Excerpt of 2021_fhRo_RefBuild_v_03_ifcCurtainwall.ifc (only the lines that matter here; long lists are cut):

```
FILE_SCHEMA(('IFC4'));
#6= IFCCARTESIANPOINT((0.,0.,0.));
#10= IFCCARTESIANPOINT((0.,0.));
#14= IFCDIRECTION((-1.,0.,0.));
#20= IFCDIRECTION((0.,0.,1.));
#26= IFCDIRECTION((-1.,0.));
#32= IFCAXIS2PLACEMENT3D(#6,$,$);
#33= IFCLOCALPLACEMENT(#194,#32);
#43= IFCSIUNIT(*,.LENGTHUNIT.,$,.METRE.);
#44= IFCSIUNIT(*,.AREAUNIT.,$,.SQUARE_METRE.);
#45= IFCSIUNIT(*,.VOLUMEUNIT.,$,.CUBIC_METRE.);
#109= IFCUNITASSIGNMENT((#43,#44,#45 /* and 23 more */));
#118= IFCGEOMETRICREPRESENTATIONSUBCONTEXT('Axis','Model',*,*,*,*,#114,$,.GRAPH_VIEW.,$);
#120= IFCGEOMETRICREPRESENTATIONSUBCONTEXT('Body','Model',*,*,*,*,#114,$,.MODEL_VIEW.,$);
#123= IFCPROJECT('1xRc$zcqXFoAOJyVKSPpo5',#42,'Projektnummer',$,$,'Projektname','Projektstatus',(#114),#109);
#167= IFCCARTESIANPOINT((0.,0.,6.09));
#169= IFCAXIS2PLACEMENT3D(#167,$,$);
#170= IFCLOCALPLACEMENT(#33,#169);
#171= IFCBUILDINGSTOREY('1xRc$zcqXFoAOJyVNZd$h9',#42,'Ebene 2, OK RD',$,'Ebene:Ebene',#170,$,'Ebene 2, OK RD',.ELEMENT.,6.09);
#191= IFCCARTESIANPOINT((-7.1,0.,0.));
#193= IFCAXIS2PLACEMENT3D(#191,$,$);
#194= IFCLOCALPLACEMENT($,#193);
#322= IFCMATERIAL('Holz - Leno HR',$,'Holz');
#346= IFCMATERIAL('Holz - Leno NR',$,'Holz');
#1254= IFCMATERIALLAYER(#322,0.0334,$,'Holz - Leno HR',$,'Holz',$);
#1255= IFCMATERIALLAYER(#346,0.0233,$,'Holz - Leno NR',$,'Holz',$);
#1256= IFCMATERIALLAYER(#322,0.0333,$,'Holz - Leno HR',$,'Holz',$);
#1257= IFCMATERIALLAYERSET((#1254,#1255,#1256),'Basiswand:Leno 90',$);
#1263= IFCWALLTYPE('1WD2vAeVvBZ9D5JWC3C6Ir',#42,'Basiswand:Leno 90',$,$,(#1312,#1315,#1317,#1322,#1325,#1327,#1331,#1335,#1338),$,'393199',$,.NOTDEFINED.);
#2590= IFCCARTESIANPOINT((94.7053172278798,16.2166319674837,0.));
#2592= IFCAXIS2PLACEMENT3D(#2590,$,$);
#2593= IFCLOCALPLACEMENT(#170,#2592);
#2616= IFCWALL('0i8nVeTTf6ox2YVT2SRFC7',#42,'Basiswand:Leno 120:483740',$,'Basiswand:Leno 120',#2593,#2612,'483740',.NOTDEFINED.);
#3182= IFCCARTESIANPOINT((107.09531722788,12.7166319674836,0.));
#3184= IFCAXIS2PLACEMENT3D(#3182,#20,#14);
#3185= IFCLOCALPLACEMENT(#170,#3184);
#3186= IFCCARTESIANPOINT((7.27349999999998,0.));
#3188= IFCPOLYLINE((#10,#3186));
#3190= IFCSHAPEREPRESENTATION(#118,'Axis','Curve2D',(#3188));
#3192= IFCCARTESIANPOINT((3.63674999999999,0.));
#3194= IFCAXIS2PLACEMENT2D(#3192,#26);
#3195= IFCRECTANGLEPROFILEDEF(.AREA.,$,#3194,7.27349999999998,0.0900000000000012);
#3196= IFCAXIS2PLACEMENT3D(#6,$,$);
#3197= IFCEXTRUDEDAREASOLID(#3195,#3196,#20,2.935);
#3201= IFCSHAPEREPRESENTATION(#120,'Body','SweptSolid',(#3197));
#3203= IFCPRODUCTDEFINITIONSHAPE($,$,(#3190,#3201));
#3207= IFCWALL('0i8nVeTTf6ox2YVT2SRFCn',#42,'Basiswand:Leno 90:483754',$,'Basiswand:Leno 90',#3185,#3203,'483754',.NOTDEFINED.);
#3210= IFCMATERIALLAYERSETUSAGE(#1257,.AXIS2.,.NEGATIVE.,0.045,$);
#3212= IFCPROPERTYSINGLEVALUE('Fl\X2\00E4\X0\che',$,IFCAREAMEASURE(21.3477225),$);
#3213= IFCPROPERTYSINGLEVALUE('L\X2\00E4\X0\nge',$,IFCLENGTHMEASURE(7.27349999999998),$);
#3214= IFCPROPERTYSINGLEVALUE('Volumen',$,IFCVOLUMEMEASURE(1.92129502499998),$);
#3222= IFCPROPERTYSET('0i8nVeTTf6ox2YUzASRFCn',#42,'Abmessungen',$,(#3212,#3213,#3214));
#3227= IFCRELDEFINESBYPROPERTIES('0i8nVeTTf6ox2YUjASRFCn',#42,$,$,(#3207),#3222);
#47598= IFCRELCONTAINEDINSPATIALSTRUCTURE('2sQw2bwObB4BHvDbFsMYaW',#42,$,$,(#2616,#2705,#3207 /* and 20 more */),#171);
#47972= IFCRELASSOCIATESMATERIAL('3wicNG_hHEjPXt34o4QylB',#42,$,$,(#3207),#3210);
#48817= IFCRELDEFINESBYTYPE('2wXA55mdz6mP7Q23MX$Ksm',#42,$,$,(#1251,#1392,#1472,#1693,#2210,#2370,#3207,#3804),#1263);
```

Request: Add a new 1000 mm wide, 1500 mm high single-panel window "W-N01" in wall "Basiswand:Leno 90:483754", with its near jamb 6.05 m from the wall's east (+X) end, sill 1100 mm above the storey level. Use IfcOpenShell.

```python
import numpy as np
import ifcopenshell
import ifcopenshell.api.feature
import ifcopenshell.api.geometry
import ifcopenshell.api.pset
import ifcopenshell.api.root
import ifcopenshell.api.spatial
import ifcopenshell.geom
import ifcopenshell.util.element
import ifcopenshell.util.placement
import ifcopenshell.util.representation
import ifcopenshell.util.shape
import ifcopenshell.util.unit

model = ifcopenshell.open("2021_fhRo_RefBuild_v_03_ifcCurtainwall.ifc")
unit_scale = ifcopenshell.util.unit.calculate_unit_scale(model)
area_scale = ifcopenshell.util.unit.calculate_unit_scale(model, "AREAUNIT")
volume_scale = ifcopenshell.util.unit.calculate_unit_scale(model, "VOLUMEUNIT")
settings = ifcopenshell.geom.settings()


def volume(element):
    """Net volume in cubic metres, openings subtracted."""
    shape = ifcopenshell.geom.create_shape(settings, element)
    return ifcopenshell.util.shape.get_volume(shape.geometry)


wall = model.by_id(3207)
storey = ifcopenshell.util.element.get_container(wall, ifc_class="IfcBuildingStorey")
context = ifcopenshell.util.representation.get_context(model, "Model", "Body", "MODEL_VIEW")
before = volume(wall)

width, height, from_end, sill = 1, 1.5, 6.05, 1.1  # metres

# The wall runs along its own X axis, and the end named is its -X end.
wall_shape = ifcopenshell.geom.create_shape(settings, wall)
x, y, z = ifcopenshell.util.shape.get_vertices(wall_shape.geometry).T
start = x.min() + from_end
face, thickness = float(y.min()), float(y.max() - y.min())
wall_matrix = ifcopenshell.util.placement.get_local_placement(wall.ObjectPlacement)
level = ifcopenshell.util.placement.get_local_placement(storey.ObjectPlacement)[2, 3]


def in_wall(x, y):
    """Placement at x, y metres in the wall's axes, at sill height."""
    matrix = wall_matrix.copy()
    matrix[:, 3] = wall_matrix @ np.array([x / unit_scale, y / unit_scale, 0.0, 1.0])
    matrix[2, 3] = level + sill / unit_scale
    return matrix


# Opening: a box that overshoots both wall faces by 50 mm.
opening = ifcopenshell.api.root.create_entity(model, ifc_class="IfcOpeningElement", predefined_type="OPENING")
box = ifcopenshell.api.geometry.add_wall_representation(
    model, context=context, length=width, height=height, thickness=thickness + 0.1
)
ifcopenshell.api.geometry.assign_representation(model, product=opening, representation=box)
ifcopenshell.api.geometry.edit_object_placement(model, product=opening, matrix=in_wall(start, face - 0.05), is_si=False)
ifcopenshell.api.feature.add_feature(model, feature=opening, element=wall)

window = ifcopenshell.api.root.create_entity(model, ifc_class="IfcWindow", name="W-N01", predefined_type="WINDOW")
window.OverallWidth, window.OverallHeight = width / unit_scale, height / unit_scale
window.PartitioningType = "SINGLE_PANEL"
body = ifcopenshell.api.geometry.add_window_representation(
    model,
    context=context,
    overall_width=window.OverallWidth,
    overall_height=window.OverallHeight,
    partition_type="SINGLE_PANEL",
)
ifcopenshell.api.geometry.assign_representation(model, product=window, representation=body)
ifcopenshell.api.spatial.assign_container(model, products=[window], relating_structure=storey)
ifcopenshell.api.feature.add_filling(model, opening=opening, element=window)

# Centre the window in the wall's thickness.
ifcopenshell.api.geometry.edit_object_placement(model, product=window, matrix=in_wall(start, face), is_si=False)
window_shape = ifcopenshell.geom.create_shape(settings, window)
depth = ifcopenshell.util.shape.get_vertices(window_shape.geometry)[:, 1]
offset = face + thickness / 2 - (depth.min() + depth.max()) / 2
ifcopenshell.api.geometry.edit_object_placement(model, product=window, matrix=in_wall(start, offset), is_si=False)

after = volume(wall)

# Update the wall's stored quantities.
pset = model.by_id(ifcopenshell.util.element.get_pset(wall, "Abmessungen", should_inherit=False)["id"])
ifcopenshell.api.pset.edit_pset(model, pset=pset, properties={
    "Fläche": model.create_entity("IfcAreaMeasure", after / thickness / area_scale),
    "Volumen": model.create_entity("IfcVolumeMeasure", after / volume_scale),
})

print(f"wall volume {before:.3f} -> {after:.3f} m3")

model.write("2021_fhRo_RefBuild_v_03_ifcCurtainwall_rev.ifc")
```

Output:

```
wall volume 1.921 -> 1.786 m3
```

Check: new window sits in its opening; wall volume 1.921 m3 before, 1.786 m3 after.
